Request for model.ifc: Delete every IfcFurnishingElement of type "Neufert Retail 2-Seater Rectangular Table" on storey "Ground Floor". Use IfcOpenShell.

First a look at what the model holds.

```python
import ifcopenshell
import ifcopenshell.util.element

model = ifcopenshell.open("model.ifc")
print(model.schema)
storey = next(s for s in model.by_type("IfcBuildingStorey") if s.Name == "Ground Floor")
furniture = [e for e in ifcopenshell.util.element.get_decomposition(storey) if e.is_a("IfcFurnishingElement")]
seen = {}
for e in furniture:
    element_type = ifcopenshell.util.element.get_type(e)
    name = element_type.Name if element_type not in (None, e) else None
    seen[name] = seen.get(name, 0) + 1
for name, count in sorted(seen.items(), key=str):
    print(count, "x", name)
```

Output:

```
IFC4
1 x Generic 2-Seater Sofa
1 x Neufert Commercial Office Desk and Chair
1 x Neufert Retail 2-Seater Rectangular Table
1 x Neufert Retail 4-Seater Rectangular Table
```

```python
import ifcopenshell
import ifcopenshell.api.root
import ifcopenshell.util.element

model = ifcopenshell.open("model.ifc")

storey = next(s for s in model.by_type("IfcBuildingStorey") if s.Name == "Ground Floor")
furniture = [e for e in ifcopenshell.util.element.get_decomposition(storey) if e.is_a("IfcFurnishingElement")]
targets = [e for e in furniture if (t := ifcopenshell.util.element.get_type(e)) not in (None, e) and t.Name == "Neufert Retail 2-Seater Rectangular Table"]

for e in targets:
    ifcopenshell.api.root.remove_product(model, product=e)
print(len(targets), "removed")

model.write("model_rev.ifc")
```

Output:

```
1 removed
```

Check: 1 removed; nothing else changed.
